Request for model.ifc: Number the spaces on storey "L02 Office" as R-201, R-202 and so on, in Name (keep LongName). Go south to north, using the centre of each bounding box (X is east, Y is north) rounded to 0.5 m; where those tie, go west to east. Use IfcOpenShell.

First a look at what the model holds.

```python
import ifcopenshell
import ifcopenshell.util.element
import ifcopenshell.util.placement

model = ifcopenshell.open("model.ifc")
print(model.schema)
storey = next(s for s in model.by_type("IfcBuildingStorey") if s.Name == "L02 Office")
spaces = [e for e in ifcopenshell.util.element.get_decomposition(storey) if e.is_a("IfcSpace")]
for e in sorted(spaces, key=lambda e: e.id()):
    origin = ifcopenshell.util.placement.get_local_placement(e.ObjectPlacement)[:3, 3]
    print(e.id(), e.Name, e.LongName, origin.round(2) + 0.0, sep=" | ")
```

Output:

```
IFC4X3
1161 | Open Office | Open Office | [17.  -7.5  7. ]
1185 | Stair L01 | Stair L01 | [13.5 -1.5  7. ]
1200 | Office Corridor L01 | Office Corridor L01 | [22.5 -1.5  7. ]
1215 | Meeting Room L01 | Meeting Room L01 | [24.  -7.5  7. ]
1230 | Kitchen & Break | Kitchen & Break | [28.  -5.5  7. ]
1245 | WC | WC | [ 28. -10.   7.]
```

```python
import ifcopenshell
import ifcopenshell.geom
import ifcopenshell.util.element
import ifcopenshell.util.shape

model = ifcopenshell.open("model.ifc")
settings = ifcopenshell.geom.settings()
settings.set("use-world-coords", True)


def centre(element):
    shape = ifcopenshell.geom.create_shape(settings, element)
    return ifcopenshell.util.shape.get_bbox_centroid(shape.geometry)


storey = next(s for s in model.by_type("IfcBuildingStorey") if s.Name == "L02 Office")
spaces = [e for e in ifcopenshell.util.element.get_decomposition(storey) if e.is_a("IfcSpace")]

# Insertion points can sit at a corner or the storey origin, so sort by the geometry (in metres).
centres = {e: centre(e) for e in spaces}
spaces.sort(key=lambda e: (round(centres[e][1] / 0.5), centres[e][0]))

for i, e in enumerate(spaces, start=1):
    number = f"R-2{i:02d}"
    e.Name = number
    print(e.id(), number)

model.write("model_edited.ifc")
```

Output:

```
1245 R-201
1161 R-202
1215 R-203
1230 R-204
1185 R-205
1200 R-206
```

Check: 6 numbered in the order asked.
